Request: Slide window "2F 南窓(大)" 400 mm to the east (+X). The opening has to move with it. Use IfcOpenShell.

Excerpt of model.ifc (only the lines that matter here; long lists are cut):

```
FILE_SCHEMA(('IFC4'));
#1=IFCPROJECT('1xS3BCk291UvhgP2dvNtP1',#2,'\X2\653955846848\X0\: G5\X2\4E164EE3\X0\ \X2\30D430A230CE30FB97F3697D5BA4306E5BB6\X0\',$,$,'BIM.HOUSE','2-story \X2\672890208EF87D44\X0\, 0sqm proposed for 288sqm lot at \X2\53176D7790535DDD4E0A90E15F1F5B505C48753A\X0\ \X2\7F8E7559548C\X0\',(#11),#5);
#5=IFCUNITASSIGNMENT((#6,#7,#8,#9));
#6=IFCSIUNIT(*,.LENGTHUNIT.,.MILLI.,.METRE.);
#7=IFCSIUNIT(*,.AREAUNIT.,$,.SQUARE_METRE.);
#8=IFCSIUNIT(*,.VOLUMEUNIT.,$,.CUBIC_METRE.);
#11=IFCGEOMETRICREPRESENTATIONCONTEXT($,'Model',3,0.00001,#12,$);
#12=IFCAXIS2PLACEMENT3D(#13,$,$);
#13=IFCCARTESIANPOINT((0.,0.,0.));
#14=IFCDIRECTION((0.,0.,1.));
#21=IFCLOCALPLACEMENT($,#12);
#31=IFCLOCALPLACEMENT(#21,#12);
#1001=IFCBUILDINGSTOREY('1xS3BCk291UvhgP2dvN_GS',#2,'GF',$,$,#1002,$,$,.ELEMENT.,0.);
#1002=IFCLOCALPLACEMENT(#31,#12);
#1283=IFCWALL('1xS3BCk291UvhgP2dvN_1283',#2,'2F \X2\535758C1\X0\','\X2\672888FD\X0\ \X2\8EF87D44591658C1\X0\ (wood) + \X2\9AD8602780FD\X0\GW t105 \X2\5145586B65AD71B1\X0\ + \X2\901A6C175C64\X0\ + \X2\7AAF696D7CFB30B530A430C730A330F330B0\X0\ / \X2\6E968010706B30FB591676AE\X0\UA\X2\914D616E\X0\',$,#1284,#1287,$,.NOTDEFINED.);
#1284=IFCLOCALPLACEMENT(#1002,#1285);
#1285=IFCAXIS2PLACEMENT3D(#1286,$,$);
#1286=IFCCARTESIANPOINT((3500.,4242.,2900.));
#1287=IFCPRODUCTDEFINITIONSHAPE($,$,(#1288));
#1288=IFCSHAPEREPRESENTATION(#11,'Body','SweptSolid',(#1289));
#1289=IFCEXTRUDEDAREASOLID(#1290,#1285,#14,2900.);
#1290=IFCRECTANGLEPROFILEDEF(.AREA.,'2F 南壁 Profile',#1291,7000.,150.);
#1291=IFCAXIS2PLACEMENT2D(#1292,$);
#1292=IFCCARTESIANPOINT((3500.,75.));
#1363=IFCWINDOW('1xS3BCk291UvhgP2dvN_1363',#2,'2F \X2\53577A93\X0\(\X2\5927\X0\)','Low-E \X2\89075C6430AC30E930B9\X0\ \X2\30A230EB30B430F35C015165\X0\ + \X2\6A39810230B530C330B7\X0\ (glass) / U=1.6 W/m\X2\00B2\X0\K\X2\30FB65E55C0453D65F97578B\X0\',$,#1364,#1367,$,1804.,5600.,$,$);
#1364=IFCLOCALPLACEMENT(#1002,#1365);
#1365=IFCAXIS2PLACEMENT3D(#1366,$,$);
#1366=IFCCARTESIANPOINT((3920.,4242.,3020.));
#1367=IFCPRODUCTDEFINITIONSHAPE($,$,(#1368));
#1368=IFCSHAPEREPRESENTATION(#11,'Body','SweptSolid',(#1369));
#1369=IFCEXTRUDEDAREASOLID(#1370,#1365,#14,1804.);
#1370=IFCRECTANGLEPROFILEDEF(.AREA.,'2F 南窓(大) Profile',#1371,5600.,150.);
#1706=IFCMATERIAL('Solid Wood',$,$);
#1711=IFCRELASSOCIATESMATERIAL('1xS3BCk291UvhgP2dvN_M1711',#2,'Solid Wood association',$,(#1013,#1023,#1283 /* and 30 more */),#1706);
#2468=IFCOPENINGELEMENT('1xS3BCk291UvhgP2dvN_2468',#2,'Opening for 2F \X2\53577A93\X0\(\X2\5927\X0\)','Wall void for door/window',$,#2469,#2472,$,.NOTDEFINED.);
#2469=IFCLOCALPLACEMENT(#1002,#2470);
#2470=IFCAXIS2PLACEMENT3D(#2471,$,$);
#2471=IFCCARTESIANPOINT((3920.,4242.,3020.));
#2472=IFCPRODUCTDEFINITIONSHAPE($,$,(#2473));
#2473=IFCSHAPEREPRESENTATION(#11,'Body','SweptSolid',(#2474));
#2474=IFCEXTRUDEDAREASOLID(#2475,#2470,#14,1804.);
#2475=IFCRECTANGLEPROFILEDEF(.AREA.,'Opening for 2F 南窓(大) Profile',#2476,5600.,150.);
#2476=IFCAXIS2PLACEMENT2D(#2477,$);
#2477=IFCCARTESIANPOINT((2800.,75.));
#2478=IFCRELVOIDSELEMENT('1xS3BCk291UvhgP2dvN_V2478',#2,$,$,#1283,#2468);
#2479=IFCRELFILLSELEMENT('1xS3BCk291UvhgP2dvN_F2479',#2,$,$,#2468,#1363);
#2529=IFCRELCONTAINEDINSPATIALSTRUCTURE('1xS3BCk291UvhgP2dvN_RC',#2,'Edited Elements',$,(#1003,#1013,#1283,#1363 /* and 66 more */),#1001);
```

```python
import ifcopenshell
import ifcopenshell.api.geometry
import ifcopenshell.util.placement

model = ifcopenshell.open("model.ifc")

window = model.by_id(1363)
opening = window.FillsVoids[0].RelatingOpeningElement
wall = opening.VoidsElements[0].RelatingBuildingElement

wall_matrix = ifcopenshell.util.placement.get_local_placement(wall.ObjectPlacement)
shift = wall_matrix[:3, 0] * 400.0
before = ifcopenshell.util.placement.get_local_placement(window.ObjectPlacement)[:3, 3].copy()

# The window is not placed relative to its opening, so move both.
for product in (opening, window):
    matrix = ifcopenshell.util.placement.get_local_placement(product.ObjectPlacement)
    matrix[:3, 3] += shift
    ifcopenshell.api.geometry.edit_object_placement(model, product=product, matrix=matrix, is_si=False)

after = ifcopenshell.util.placement.get_local_placement(window.ObjectPlacement)[:3, 3]
print("window moved by", (after - before).round(3) + 0.0)

model.write("model-out.ifc")
```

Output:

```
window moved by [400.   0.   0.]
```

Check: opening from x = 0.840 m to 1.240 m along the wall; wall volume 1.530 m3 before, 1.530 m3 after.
